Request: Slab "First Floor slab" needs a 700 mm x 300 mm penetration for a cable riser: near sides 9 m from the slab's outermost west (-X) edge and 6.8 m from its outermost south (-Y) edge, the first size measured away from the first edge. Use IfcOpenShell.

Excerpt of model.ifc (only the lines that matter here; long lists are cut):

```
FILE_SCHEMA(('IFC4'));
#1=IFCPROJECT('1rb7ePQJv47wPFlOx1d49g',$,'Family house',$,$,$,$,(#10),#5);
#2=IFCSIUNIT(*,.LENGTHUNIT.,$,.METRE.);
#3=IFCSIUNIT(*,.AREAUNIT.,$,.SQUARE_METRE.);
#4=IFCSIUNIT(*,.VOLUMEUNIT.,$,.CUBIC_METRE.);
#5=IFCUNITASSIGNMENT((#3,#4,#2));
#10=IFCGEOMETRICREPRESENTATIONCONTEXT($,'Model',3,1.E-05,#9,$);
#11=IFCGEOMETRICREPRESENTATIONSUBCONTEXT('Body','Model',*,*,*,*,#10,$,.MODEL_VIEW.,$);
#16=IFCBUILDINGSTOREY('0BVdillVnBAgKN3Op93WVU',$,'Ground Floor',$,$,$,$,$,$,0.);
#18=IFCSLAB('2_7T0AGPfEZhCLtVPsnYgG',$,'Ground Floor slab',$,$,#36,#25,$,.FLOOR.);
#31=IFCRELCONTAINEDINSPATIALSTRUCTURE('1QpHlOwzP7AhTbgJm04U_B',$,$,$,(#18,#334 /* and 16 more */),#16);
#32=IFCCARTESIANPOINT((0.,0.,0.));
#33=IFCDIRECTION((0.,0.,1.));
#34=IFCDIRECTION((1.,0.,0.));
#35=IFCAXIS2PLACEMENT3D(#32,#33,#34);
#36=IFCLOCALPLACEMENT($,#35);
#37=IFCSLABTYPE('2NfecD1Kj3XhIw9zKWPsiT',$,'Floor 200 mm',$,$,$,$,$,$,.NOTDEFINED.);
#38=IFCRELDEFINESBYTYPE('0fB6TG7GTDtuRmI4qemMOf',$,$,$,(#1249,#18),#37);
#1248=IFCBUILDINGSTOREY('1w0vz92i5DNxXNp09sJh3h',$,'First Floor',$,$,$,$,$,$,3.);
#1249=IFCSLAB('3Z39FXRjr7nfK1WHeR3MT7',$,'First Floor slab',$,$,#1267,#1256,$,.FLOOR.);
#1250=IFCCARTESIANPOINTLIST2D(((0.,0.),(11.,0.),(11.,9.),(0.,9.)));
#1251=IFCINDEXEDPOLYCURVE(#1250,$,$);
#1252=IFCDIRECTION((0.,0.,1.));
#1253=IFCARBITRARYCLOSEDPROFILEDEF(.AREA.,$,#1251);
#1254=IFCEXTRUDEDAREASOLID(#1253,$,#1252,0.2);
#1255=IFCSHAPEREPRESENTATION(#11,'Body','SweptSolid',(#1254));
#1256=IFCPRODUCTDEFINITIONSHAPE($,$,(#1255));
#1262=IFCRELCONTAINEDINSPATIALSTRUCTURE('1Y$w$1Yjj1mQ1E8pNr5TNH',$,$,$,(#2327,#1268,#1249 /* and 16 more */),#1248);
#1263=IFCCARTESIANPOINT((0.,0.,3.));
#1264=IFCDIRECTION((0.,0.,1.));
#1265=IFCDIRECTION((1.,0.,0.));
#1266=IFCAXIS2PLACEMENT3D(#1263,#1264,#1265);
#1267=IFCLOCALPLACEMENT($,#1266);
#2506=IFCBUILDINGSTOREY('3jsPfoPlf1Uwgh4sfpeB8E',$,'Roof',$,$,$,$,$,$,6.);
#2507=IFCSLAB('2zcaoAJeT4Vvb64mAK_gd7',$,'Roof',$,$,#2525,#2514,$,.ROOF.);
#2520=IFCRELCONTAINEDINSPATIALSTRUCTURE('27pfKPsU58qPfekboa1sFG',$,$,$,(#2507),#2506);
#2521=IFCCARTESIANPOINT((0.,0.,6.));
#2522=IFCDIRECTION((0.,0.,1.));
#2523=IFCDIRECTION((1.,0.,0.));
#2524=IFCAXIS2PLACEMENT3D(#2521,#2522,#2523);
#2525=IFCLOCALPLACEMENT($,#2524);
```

```python
import numpy as np
import ifcopenshell
import ifcopenshell.api.feature
import ifcopenshell.api.geometry
import ifcopenshell.api.root
import ifcopenshell.geom
import ifcopenshell.util.placement
import ifcopenshell.util.representation
import ifcopenshell.util.shape
import ifcopenshell.util.unit

model = ifcopenshell.open("model.ifc")
unit_scale = ifcopenshell.util.unit.calculate_unit_scale(model)
settings = ifcopenshell.geom.settings()


def volume(element):
    """Net volume in cubic metres, openings subtracted."""
    shape = ifcopenshell.geom.create_shape(settings, element)
    return ifcopenshell.util.shape.get_volume(shape.geometry)


slab = model.by_guid("3Z39FXRjr7nfK1WHeR3MT7")
before = volume(slab)

# Extent in the slab's own axes, in metres. The edges named are its -X and -Y sides.
slab_shape = ifcopenshell.geom.create_shape(settings, slab)
vertices = ifcopenshell.util.shape.get_vertices(slab_shape.geometry)
x_min, y_min, bottom = vertices.min(axis=0)
top = vertices[:, 2].max()

opening = ifcopenshell.api.root.create_entity(model, ifc_class="IfcOpeningElement", name="Cable riser opening", predefined_type="OPENING")
context = ifcopenshell.util.representation.get_context(model, "Model", "Body", "MODEL_VIEW")
width, depth = 0.7, 0.3
outline = [(0.0, 0.0), (width, 0.0), (width, depth), (0.0, depth), (0.0, 0.0)]
# Overshoot both faces by 50 mm so the cut is clean.
shape = ifcopenshell.api.geometry.add_slab_representation(
    model, context=context, depth=top - bottom + 0.1, polyline=outline
)
ifcopenshell.api.geometry.assign_representation(model, product=opening, representation=shape)

matrix = ifcopenshell.util.placement.get_local_placement(slab.ObjectPlacement)
matrix[:, 3] = matrix @ np.append(np.array([x_min + 9, y_min + 6.8, bottom - 0.05]) / unit_scale, 1.0)
ifcopenshell.api.geometry.edit_object_placement(model, product=opening, matrix=matrix, is_si=False)
ifcopenshell.api.feature.add_feature(model, feature=opening, element=slab)

after = volume(slab)

print(f"slab volume {before:.3f} -> {after:.3f} m3")

model.write("model_updated.ifc")
```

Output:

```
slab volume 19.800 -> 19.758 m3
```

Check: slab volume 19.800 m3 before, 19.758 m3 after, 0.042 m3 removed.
